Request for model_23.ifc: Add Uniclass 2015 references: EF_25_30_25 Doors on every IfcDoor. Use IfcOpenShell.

First a look at what the model holds.

```python
import ifcopenshell

model = ifcopenshell.open("model_23.ifc")
print(model.schema)
print("classifications:", [c.Name for c in model.by_type("IfcClassification")])
for ifc_class in ("IfcDoor", "IfcRoof", "IfcStair", "IfcWall", "IfcWindow"):
    print(ifc_class, len(model.by_type(ifc_class)))
```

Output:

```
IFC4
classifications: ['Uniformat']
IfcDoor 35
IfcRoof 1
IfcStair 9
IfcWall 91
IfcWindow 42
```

```python
import ifcopenshell
import ifcopenshell.api.classification

model = ifcopenshell.open("model_23.ifc")

system = ifcopenshell.api.classification.add_classification(model, classification="Uniclass 2015")

codes = {
    "IfcDoor": ("EF_25_30_25", "Doors"),
}
for ifc_class, (code, name) in codes.items():
    products = model.by_type(ifc_class)
    ifcopenshell.api.classification.add_reference(
        model, products=products, classification=system, identification=code, name=name
    )
    print(code, len(products))

model.write("model_23_updated.ifc")
```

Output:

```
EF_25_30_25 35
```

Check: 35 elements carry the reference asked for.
